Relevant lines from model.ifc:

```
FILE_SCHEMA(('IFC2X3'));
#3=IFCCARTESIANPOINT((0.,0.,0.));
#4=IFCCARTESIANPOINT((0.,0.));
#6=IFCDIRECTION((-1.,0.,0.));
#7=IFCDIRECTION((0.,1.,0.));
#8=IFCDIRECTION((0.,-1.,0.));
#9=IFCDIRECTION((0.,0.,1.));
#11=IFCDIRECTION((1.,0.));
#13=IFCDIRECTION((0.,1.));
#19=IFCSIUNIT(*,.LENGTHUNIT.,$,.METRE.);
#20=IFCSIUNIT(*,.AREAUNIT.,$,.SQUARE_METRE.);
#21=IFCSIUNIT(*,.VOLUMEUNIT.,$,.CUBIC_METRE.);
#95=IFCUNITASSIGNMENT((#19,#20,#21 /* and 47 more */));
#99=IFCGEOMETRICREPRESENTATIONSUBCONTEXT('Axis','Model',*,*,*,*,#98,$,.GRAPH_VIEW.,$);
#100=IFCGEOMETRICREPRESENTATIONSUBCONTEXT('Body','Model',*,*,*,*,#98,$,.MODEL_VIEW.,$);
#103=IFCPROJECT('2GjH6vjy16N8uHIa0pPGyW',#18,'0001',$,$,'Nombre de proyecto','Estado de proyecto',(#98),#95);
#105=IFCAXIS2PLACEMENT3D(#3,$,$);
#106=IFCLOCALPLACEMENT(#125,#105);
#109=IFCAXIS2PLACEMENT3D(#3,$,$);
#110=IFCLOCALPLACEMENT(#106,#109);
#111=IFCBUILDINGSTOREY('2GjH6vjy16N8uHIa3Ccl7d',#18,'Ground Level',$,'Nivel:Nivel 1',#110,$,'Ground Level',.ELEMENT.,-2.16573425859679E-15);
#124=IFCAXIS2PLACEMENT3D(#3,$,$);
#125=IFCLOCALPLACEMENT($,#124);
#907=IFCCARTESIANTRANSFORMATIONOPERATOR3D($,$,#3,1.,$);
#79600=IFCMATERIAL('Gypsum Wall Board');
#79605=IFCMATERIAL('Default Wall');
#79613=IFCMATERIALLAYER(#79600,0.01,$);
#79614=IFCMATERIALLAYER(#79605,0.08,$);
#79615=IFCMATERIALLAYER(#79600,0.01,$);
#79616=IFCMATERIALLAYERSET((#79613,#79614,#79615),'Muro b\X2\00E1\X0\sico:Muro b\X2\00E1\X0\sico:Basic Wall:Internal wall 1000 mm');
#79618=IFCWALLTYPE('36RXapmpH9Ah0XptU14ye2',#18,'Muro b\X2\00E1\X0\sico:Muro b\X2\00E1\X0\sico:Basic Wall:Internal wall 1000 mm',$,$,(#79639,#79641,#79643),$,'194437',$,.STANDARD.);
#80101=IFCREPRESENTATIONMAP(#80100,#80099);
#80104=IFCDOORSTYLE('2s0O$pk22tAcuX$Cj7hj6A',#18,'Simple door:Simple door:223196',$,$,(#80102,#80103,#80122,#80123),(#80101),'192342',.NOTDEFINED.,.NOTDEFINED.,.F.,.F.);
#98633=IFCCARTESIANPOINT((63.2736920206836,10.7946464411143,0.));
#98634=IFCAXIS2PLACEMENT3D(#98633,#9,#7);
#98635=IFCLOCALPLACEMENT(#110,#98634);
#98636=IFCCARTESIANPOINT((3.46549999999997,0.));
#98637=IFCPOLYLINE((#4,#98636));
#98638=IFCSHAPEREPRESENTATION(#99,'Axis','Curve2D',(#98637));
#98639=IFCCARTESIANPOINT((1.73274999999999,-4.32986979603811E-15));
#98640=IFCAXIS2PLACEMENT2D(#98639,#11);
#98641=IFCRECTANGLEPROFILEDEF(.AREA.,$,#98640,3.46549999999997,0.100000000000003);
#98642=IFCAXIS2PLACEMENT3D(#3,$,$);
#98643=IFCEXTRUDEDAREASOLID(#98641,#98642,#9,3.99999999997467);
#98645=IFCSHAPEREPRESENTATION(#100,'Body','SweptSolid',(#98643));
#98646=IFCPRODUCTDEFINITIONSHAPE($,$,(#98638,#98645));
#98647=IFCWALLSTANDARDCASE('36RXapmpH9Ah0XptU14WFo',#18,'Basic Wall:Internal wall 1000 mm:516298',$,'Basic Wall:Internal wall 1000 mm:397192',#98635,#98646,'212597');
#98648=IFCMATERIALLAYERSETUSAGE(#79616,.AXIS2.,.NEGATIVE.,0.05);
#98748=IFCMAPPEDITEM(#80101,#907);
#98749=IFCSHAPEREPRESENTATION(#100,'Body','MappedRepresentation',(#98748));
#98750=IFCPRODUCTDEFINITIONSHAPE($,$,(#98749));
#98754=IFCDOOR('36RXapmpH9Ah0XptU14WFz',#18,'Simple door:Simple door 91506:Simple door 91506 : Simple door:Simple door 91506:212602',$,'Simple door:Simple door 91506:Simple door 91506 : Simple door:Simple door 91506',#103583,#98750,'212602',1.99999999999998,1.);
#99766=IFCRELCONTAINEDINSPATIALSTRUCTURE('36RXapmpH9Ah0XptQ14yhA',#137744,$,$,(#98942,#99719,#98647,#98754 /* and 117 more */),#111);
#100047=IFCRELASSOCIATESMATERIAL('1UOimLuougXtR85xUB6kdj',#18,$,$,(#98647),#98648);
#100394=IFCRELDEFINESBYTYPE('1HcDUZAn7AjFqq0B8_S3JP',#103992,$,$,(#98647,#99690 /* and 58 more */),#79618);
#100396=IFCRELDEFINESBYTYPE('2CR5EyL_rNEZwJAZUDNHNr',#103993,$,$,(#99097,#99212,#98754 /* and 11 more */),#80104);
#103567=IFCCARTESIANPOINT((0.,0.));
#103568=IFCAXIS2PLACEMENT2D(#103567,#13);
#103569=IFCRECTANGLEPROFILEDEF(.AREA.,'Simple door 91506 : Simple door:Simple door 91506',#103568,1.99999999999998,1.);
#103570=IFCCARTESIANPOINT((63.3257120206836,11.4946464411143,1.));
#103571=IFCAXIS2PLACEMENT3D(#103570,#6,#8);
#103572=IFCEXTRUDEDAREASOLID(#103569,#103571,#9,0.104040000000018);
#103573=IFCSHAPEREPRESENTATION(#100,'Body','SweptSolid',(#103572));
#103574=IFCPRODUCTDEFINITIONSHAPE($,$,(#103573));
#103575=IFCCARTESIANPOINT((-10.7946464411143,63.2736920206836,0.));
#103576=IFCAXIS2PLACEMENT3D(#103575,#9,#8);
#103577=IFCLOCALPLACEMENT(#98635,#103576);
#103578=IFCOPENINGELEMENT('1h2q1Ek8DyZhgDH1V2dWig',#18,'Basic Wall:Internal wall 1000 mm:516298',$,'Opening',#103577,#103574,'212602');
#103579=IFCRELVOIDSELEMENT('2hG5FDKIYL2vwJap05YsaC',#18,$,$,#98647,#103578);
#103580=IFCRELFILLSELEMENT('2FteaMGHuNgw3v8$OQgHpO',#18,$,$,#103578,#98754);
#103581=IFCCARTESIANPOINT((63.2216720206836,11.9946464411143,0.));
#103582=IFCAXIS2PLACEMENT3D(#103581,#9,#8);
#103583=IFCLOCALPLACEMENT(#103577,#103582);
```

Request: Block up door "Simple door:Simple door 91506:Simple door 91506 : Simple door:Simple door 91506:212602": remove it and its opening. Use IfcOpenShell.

```python
import ifcopenshell
import ifcopenshell.api.feature
import ifcopenshell.api.root
import ifcopenshell.geom
import ifcopenshell.util.shape

model = ifcopenshell.open("model.ifc")
settings = ifcopenshell.geom.settings()


def volume(element):
    """Net volume in cubic metres, openings subtracted."""
    shape = ifcopenshell.geom.create_shape(settings, element)
    return ifcopenshell.util.shape.get_volume(shape.geometry)


door = model.by_guid("36RXapmpH9Ah0XptU14WFz")
opening = door.FillsVoids[0].RelatingOpeningElement
wall = opening.VoidsElements[0].RelatingBuildingElement
before = volume(wall)

ifcopenshell.api.root.remove_product(model, product=door)
ifcopenshell.api.feature.remove_feature(model, feature=opening)

after = volume(wall)

print(f"wall volume {before:.3f} -> {after:.3f} m3")

model.write("model_v2.ifc")
```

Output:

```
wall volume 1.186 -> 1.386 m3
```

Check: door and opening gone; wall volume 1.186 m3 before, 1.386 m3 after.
